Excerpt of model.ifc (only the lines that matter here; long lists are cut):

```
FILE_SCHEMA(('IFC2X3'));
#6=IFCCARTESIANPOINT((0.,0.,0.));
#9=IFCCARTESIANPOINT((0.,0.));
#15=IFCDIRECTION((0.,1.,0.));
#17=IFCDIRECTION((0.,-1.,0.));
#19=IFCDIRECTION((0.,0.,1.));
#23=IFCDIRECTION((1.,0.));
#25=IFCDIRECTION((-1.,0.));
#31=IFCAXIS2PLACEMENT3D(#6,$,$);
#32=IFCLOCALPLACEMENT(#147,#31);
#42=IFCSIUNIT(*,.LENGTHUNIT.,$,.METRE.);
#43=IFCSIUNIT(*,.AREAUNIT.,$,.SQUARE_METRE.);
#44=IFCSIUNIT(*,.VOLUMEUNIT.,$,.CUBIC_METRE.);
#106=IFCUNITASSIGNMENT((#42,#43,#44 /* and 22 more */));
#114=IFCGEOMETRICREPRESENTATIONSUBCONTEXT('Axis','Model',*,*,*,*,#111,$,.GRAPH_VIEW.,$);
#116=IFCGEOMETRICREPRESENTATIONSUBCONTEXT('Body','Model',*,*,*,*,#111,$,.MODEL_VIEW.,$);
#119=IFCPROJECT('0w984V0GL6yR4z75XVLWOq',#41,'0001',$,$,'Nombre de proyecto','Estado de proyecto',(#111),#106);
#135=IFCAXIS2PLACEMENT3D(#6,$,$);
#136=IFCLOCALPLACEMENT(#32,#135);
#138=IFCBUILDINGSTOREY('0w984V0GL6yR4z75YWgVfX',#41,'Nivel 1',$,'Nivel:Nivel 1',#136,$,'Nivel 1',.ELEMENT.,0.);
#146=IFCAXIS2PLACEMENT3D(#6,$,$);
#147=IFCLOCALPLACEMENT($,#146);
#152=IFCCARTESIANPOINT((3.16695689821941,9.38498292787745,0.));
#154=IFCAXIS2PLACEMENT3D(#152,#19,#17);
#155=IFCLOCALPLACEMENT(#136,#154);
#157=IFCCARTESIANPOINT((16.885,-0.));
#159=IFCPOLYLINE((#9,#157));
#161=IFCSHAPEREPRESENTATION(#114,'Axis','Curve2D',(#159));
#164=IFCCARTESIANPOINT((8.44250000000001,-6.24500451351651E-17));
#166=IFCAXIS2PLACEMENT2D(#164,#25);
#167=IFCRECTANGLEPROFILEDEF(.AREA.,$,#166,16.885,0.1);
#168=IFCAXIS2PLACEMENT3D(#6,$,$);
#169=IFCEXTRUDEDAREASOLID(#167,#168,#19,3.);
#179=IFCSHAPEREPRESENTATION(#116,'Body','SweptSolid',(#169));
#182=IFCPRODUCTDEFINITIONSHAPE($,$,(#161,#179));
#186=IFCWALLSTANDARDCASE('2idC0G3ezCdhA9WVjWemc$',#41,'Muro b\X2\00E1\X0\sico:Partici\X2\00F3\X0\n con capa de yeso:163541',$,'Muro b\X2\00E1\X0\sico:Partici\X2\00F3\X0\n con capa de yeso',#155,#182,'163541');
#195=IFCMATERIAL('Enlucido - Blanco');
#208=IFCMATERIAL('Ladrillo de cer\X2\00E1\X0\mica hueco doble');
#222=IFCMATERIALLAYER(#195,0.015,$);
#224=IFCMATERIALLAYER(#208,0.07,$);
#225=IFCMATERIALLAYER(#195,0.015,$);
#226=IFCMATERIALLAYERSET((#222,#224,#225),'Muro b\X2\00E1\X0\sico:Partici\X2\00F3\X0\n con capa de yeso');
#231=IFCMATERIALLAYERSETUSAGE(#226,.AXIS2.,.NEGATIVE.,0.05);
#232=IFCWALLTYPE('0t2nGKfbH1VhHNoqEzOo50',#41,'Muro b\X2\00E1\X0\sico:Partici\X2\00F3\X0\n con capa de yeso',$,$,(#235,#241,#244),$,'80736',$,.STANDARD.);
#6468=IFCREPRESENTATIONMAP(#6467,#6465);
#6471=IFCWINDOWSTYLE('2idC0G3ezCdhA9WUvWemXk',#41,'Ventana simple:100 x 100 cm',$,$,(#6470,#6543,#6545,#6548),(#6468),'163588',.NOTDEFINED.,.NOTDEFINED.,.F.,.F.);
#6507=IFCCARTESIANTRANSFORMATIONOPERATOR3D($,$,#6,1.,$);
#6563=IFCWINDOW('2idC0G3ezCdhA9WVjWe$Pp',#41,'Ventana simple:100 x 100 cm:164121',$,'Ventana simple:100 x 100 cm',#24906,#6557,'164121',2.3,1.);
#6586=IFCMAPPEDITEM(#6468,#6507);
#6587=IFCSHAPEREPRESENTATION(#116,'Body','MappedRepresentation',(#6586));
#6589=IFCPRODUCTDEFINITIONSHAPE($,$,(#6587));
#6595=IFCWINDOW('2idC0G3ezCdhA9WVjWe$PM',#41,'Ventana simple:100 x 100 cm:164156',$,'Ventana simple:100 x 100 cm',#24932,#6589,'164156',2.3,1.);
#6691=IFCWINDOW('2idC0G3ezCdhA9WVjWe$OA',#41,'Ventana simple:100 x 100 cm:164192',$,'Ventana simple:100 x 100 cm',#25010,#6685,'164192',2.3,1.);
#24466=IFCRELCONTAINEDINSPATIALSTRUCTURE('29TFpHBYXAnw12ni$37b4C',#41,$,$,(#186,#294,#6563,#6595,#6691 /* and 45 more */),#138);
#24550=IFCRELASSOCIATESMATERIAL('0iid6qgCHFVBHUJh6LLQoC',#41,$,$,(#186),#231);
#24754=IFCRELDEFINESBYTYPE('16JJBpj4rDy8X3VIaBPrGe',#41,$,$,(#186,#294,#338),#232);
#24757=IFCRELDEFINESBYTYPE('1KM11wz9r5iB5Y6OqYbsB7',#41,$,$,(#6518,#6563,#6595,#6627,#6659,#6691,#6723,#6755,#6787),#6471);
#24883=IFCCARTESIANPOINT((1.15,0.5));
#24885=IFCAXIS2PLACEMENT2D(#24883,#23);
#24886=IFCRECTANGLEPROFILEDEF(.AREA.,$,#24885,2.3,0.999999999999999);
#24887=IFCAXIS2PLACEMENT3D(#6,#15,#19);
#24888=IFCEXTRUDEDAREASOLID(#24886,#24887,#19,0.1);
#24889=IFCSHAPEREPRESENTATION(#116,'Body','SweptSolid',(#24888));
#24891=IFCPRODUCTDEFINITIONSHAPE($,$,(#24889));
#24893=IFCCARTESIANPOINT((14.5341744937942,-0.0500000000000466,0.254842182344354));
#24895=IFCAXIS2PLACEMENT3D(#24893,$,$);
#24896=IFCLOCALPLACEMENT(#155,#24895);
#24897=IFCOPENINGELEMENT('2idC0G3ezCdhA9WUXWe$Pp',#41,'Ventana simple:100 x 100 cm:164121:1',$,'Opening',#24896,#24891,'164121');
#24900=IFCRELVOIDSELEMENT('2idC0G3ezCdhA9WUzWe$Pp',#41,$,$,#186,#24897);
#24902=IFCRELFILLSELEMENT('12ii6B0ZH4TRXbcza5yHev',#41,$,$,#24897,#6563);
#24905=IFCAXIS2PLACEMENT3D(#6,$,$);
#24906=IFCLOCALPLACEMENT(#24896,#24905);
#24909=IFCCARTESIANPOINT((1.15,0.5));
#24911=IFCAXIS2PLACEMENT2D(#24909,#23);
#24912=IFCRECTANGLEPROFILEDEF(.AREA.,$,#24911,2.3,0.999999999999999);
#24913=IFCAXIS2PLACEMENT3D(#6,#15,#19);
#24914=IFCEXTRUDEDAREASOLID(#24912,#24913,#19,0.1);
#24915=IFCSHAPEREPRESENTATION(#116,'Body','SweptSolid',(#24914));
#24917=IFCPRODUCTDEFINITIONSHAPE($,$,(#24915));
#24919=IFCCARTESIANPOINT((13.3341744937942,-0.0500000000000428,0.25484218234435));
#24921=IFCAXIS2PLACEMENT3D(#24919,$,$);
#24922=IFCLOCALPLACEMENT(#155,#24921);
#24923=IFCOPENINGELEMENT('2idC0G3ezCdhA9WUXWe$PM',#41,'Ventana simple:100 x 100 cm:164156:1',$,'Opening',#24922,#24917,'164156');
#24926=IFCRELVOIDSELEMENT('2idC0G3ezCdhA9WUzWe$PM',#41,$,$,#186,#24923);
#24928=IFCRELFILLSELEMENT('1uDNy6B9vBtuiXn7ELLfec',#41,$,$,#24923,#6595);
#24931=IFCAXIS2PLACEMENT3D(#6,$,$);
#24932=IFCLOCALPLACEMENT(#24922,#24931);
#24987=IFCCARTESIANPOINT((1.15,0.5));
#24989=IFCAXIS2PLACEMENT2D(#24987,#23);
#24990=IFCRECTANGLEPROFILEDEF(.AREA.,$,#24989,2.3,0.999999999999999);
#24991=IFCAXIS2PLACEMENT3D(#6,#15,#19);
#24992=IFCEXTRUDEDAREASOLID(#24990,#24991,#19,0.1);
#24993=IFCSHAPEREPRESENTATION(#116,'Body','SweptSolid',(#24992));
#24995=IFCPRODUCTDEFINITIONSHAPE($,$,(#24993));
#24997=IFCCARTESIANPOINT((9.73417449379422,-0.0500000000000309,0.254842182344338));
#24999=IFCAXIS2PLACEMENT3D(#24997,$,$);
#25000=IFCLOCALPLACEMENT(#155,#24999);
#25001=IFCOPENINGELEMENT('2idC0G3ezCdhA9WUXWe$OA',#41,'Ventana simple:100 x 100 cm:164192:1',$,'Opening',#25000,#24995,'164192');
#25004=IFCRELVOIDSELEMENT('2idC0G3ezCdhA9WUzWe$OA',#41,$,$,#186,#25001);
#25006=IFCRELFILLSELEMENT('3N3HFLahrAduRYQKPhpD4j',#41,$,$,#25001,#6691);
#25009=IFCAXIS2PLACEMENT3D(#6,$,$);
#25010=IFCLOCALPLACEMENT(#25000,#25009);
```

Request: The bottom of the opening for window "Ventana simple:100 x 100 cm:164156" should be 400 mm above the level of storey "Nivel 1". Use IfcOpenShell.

```python
import numpy as np
import ifcopenshell
import ifcopenshell.api.geometry
import ifcopenshell.geom
import ifcopenshell.util.element
import ifcopenshell.util.placement
import ifcopenshell.util.shape
import ifcopenshell.util.unit

model = ifcopenshell.open("model.ifc")
unit_scale = ifcopenshell.util.unit.calculate_unit_scale(model)

window = model.by_guid("2idC0G3ezCdhA9WVjWe$PM")
opening = window.FillsVoids[0].RelatingOpeningElement
storey = ifcopenshell.util.element.get_container(window, ifc_class="IfcBuildingStorey")
level = ifcopenshell.util.placement.get_local_placement(storey.ObjectPlacement)[2, 3]

# The opening's origin need not be at the sill, so measure its lowest point.
shape = ifcopenshell.geom.create_shape(ifcopenshell.geom.settings(), opening)
bottom = ifcopenshell.util.shape.get_shape_bottom_elevation(shape, shape.geometry) / unit_scale
dz = level + 0.4 / unit_scale - bottom

shift = np.array([0.0, 0.0, dz])
# The window is placed relative to its opening, so it follows when the opening moves.
matrix = ifcopenshell.util.placement.get_local_placement(opening.ObjectPlacement)
matrix[:3, 3] += shift
ifcopenshell.api.geometry.edit_object_placement(
    model, product=opening, matrix=matrix, is_si=False, should_transform_children=True
)

print(f"moved by {dz * unit_scale:+.3f} m")

model.write("model-out.ifc")
```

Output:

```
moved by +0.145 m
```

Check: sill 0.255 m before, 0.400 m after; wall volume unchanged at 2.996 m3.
